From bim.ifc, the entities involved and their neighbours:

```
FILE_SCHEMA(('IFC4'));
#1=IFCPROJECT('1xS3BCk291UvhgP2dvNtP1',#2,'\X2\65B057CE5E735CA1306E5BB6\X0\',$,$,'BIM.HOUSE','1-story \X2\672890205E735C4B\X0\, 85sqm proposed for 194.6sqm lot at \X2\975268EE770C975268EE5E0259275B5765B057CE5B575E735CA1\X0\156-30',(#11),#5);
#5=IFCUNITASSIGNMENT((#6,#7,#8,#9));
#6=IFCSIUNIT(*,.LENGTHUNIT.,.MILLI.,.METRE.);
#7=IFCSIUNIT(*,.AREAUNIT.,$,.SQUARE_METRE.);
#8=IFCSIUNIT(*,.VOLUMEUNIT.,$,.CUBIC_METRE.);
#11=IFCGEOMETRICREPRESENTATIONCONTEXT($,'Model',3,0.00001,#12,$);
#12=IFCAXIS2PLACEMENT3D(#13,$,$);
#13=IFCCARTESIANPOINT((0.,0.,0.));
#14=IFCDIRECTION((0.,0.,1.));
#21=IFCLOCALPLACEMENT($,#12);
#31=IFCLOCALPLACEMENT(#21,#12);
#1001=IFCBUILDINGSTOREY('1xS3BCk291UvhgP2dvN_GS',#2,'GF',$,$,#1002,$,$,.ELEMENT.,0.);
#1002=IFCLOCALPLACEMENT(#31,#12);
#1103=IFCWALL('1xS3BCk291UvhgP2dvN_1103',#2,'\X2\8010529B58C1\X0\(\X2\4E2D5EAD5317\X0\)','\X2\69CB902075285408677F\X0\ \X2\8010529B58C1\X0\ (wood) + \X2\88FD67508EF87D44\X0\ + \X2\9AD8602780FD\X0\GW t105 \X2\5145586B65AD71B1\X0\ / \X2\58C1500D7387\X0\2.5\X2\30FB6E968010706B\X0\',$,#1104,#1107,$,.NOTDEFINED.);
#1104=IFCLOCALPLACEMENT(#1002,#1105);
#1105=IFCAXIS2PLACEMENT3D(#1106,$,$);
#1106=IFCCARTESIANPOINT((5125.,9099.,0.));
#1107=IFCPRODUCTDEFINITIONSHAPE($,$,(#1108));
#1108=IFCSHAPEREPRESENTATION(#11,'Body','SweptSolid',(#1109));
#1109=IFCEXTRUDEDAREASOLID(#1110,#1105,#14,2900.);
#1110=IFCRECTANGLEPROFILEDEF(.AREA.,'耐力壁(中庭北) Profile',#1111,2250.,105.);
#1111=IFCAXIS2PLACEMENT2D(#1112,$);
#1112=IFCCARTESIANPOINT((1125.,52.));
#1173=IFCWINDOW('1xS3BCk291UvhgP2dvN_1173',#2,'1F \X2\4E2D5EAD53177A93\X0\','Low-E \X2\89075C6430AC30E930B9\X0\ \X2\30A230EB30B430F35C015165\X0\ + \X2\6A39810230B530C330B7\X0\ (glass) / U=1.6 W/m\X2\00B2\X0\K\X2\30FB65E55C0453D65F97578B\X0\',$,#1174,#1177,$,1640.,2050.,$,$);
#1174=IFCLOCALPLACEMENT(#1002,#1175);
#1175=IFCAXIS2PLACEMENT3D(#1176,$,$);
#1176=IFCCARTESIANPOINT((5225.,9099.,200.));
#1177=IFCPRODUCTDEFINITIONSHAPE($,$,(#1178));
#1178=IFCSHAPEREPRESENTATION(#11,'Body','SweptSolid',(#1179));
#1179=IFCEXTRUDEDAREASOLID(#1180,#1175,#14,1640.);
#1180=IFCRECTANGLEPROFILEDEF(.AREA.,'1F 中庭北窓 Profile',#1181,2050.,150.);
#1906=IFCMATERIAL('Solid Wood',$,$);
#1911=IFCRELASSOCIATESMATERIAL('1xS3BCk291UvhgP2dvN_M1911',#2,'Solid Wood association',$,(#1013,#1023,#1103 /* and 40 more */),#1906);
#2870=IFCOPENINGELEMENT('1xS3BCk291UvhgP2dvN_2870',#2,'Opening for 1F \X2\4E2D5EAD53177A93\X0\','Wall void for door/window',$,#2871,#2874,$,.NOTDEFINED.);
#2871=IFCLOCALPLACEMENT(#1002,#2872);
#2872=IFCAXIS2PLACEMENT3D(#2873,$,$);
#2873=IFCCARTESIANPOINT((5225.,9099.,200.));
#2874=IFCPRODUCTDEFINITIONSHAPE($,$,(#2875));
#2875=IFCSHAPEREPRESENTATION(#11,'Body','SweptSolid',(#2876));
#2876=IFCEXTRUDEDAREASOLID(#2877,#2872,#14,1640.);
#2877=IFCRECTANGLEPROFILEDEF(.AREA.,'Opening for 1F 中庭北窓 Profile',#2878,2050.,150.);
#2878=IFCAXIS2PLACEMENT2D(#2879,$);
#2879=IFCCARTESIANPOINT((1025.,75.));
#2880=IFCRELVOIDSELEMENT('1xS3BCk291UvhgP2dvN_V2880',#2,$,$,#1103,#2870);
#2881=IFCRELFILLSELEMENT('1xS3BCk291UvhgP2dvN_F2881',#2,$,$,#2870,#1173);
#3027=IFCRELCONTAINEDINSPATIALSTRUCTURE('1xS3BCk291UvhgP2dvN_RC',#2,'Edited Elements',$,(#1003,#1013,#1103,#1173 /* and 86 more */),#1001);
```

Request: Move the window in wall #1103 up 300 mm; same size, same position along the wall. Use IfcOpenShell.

```python
import numpy as np
import ifcopenshell
import ifcopenshell.api.geometry
import ifcopenshell.util.placement
import ifcopenshell.util.unit

model = ifcopenshell.open("bim.ifc")
unit_scale = ifcopenshell.util.unit.calculate_unit_scale(model)

window = model.by_guid("1xS3BCk291UvhgP2dvN_1173")
opening = window.FillsVoids[0].RelatingOpeningElement
dz = 0.3 / unit_scale

shift = np.array([0.0, 0.0, dz])
# The window is not placed relative to its opening, so move both.
for product in (opening, window):
    matrix = ifcopenshell.util.placement.get_local_placement(product.ObjectPlacement)
    matrix[:3, 3] += shift
    ifcopenshell.api.geometry.edit_object_placement(model, product=product, matrix=matrix, is_si=False)

print(f"moved by {dz * unit_scale:+.3f} m")

model.write("bim_v2.ifc")
```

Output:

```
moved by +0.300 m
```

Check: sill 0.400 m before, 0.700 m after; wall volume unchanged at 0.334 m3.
